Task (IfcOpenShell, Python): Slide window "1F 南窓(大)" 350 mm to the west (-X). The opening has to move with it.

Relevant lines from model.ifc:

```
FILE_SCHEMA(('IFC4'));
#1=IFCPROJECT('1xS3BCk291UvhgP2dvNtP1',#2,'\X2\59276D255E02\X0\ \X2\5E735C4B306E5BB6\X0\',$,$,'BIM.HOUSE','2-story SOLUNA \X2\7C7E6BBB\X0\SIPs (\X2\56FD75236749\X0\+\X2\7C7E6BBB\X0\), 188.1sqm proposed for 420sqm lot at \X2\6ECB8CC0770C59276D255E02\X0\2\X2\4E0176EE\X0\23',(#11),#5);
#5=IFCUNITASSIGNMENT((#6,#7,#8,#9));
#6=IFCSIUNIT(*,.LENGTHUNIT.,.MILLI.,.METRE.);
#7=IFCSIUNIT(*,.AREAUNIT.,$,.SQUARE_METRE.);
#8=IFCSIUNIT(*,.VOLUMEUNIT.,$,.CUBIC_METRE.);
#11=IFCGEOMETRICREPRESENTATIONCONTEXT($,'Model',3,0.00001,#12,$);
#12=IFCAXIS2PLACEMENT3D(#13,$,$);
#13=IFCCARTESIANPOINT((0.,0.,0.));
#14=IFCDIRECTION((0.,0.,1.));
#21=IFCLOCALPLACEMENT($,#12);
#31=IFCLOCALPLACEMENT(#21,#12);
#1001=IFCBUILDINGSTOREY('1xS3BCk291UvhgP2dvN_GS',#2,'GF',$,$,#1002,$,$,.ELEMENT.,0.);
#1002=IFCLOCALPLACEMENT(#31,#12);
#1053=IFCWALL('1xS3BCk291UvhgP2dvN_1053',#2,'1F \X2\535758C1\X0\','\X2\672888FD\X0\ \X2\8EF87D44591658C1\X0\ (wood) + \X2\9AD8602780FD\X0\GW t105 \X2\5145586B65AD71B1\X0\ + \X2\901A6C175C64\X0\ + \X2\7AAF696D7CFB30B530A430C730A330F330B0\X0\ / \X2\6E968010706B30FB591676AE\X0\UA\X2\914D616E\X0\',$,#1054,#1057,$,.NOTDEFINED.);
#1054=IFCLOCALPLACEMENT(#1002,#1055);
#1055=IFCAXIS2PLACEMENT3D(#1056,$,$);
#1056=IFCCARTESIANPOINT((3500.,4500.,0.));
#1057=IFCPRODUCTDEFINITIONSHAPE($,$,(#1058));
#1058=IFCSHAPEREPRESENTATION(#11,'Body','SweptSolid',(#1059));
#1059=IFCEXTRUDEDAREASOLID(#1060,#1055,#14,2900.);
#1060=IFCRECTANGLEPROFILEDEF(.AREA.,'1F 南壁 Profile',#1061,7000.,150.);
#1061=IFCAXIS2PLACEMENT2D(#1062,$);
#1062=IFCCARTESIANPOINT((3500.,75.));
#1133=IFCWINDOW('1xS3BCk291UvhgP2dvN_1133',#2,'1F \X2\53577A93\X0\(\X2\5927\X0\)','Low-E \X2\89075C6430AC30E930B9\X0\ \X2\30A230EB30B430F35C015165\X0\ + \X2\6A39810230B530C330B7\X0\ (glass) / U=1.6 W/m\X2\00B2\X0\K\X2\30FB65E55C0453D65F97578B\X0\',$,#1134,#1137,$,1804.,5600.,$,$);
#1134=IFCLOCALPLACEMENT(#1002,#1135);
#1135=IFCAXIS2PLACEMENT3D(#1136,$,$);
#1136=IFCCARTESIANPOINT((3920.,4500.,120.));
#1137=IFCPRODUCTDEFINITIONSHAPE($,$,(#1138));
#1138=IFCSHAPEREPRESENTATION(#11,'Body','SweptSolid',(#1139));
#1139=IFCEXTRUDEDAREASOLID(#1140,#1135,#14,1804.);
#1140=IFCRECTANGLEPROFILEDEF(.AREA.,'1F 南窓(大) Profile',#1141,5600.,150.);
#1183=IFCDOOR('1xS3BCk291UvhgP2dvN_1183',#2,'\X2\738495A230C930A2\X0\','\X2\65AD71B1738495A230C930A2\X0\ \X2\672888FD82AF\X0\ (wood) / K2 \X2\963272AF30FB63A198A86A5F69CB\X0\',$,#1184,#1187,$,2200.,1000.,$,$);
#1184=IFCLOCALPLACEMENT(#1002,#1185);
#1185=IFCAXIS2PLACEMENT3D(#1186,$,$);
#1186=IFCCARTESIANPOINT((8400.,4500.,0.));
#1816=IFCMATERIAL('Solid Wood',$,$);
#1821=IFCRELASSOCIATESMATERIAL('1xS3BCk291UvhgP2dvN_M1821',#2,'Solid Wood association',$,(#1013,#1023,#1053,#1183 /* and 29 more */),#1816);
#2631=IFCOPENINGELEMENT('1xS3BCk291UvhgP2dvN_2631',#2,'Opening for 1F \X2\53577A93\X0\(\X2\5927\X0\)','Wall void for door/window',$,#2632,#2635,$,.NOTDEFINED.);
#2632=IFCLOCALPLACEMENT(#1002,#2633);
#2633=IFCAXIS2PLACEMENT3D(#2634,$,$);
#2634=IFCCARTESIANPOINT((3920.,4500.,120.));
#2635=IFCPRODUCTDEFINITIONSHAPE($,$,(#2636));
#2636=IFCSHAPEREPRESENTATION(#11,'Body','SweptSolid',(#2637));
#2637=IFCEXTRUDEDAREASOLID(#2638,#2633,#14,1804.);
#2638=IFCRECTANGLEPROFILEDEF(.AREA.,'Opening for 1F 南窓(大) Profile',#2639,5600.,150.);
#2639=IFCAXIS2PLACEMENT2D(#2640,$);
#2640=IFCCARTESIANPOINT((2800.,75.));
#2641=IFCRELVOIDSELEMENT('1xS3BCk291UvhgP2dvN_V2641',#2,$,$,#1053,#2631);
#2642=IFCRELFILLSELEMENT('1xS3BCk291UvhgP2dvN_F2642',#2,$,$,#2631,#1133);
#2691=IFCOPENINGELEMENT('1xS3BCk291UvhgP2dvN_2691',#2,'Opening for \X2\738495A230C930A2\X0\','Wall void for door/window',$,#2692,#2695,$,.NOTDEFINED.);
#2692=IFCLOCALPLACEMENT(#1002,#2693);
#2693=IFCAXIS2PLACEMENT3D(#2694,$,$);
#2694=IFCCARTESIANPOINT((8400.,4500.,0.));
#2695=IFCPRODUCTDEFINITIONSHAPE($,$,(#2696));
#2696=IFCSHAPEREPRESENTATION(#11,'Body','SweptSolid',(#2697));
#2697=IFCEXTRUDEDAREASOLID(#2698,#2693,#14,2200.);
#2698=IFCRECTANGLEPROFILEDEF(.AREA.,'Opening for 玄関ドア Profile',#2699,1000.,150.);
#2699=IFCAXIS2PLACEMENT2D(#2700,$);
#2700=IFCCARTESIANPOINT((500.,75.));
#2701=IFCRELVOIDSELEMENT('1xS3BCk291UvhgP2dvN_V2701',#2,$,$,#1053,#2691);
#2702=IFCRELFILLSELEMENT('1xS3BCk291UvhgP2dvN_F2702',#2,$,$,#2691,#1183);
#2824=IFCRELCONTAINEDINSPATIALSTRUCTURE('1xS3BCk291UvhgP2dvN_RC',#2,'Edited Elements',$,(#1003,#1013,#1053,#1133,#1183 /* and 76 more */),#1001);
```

```python
import ifcopenshell
import ifcopenshell.api.geometry
import ifcopenshell.util.placement
import ifcopenshell.util.unit

model = ifcopenshell.open("model.ifc")
unit_scale = ifcopenshell.util.unit.calculate_unit_scale(model)

window = model.by_guid("1xS3BCk291UvhgP2dvN_1133")
opening = window.FillsVoids[0].RelatingOpeningElement
wall = opening.VoidsElements[0].RelatingBuildingElement

wall_matrix = ifcopenshell.util.placement.get_local_placement(wall.ObjectPlacement)
shift = wall_matrix[:3, 0] * -0.35 / unit_scale
before = ifcopenshell.util.placement.get_local_placement(window.ObjectPlacement)[:3, 3].copy()

# The window is not placed relative to its opening, so move both.
for product in (opening, window):
    matrix = ifcopenshell.util.placement.get_local_placement(product.ObjectPlacement)
    matrix[:3, 3] += shift
    ifcopenshell.api.geometry.edit_object_placement(model, product=product, matrix=matrix, is_si=False)

after = ifcopenshell.util.placement.get_local_placement(window.ObjectPlacement)[:3, 3]
print("window moved by", (after - before).round(3) + 0.0)

model.write("model-out.ifc")
```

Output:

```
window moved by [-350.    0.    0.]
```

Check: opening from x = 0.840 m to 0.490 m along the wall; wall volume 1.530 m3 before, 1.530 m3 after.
